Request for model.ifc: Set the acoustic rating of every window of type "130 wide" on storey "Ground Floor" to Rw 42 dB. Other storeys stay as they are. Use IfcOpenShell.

First a look at what the model holds.

```python
import ifcopenshell
import ifcopenshell.util.element

model = ifcopenshell.open("model.ifc")
print(model.schema)
storey = next(s for s in model.by_type("IfcBuildingStorey") if s.Name == "Ground Floor")
windows = [e for e in ifcopenshell.util.element.get_decomposition(storey) if e.is_a("IfcWindow")]
seen = {}
for e in windows:
    element_type = ifcopenshell.util.element.get_type(e)
    key = (element_type.Name if element_type != e and element_type else None, ifcopenshell.util.element.get_pset(e, "Pset_WindowCommon", "AcousticRating"))
    seen[key] = seen.get(key, 0) + 1
for (name, value), count in sorted(seen.items(), key=str):
    print(count, "x", name, "|", value)
```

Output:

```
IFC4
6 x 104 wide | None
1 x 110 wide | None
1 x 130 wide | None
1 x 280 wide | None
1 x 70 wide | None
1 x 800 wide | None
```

```python
import ifcopenshell
import ifcopenshell.api.pset
import ifcopenshell.util.element

model = ifcopenshell.open("model.ifc")

storey = next(s for s in model.by_type("IfcBuildingStorey") if s.Name == "Ground Floor")
windows = [e for e in ifcopenshell.util.element.get_decomposition(storey) if e.is_a("IfcWindow")]

count = 0
for e in windows:
    element_type = ifcopenshell.util.element.get_type(e)
    if element_type in (None, e) or element_type.Name != "130 wide":
        continue
    # add_pset returns the element's existing set when there is one.
    pset = ifcopenshell.api.pset.add_pset(model, product=e, name="Pset_WindowCommon")
    ifcopenshell.api.pset.edit_pset(model, pset=pset, properties={"AcousticRating": "Rw 42 dB"})
    count += 1

print(count, "windows updated")

model.write("model_updated.ifc")
```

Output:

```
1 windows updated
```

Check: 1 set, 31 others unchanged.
